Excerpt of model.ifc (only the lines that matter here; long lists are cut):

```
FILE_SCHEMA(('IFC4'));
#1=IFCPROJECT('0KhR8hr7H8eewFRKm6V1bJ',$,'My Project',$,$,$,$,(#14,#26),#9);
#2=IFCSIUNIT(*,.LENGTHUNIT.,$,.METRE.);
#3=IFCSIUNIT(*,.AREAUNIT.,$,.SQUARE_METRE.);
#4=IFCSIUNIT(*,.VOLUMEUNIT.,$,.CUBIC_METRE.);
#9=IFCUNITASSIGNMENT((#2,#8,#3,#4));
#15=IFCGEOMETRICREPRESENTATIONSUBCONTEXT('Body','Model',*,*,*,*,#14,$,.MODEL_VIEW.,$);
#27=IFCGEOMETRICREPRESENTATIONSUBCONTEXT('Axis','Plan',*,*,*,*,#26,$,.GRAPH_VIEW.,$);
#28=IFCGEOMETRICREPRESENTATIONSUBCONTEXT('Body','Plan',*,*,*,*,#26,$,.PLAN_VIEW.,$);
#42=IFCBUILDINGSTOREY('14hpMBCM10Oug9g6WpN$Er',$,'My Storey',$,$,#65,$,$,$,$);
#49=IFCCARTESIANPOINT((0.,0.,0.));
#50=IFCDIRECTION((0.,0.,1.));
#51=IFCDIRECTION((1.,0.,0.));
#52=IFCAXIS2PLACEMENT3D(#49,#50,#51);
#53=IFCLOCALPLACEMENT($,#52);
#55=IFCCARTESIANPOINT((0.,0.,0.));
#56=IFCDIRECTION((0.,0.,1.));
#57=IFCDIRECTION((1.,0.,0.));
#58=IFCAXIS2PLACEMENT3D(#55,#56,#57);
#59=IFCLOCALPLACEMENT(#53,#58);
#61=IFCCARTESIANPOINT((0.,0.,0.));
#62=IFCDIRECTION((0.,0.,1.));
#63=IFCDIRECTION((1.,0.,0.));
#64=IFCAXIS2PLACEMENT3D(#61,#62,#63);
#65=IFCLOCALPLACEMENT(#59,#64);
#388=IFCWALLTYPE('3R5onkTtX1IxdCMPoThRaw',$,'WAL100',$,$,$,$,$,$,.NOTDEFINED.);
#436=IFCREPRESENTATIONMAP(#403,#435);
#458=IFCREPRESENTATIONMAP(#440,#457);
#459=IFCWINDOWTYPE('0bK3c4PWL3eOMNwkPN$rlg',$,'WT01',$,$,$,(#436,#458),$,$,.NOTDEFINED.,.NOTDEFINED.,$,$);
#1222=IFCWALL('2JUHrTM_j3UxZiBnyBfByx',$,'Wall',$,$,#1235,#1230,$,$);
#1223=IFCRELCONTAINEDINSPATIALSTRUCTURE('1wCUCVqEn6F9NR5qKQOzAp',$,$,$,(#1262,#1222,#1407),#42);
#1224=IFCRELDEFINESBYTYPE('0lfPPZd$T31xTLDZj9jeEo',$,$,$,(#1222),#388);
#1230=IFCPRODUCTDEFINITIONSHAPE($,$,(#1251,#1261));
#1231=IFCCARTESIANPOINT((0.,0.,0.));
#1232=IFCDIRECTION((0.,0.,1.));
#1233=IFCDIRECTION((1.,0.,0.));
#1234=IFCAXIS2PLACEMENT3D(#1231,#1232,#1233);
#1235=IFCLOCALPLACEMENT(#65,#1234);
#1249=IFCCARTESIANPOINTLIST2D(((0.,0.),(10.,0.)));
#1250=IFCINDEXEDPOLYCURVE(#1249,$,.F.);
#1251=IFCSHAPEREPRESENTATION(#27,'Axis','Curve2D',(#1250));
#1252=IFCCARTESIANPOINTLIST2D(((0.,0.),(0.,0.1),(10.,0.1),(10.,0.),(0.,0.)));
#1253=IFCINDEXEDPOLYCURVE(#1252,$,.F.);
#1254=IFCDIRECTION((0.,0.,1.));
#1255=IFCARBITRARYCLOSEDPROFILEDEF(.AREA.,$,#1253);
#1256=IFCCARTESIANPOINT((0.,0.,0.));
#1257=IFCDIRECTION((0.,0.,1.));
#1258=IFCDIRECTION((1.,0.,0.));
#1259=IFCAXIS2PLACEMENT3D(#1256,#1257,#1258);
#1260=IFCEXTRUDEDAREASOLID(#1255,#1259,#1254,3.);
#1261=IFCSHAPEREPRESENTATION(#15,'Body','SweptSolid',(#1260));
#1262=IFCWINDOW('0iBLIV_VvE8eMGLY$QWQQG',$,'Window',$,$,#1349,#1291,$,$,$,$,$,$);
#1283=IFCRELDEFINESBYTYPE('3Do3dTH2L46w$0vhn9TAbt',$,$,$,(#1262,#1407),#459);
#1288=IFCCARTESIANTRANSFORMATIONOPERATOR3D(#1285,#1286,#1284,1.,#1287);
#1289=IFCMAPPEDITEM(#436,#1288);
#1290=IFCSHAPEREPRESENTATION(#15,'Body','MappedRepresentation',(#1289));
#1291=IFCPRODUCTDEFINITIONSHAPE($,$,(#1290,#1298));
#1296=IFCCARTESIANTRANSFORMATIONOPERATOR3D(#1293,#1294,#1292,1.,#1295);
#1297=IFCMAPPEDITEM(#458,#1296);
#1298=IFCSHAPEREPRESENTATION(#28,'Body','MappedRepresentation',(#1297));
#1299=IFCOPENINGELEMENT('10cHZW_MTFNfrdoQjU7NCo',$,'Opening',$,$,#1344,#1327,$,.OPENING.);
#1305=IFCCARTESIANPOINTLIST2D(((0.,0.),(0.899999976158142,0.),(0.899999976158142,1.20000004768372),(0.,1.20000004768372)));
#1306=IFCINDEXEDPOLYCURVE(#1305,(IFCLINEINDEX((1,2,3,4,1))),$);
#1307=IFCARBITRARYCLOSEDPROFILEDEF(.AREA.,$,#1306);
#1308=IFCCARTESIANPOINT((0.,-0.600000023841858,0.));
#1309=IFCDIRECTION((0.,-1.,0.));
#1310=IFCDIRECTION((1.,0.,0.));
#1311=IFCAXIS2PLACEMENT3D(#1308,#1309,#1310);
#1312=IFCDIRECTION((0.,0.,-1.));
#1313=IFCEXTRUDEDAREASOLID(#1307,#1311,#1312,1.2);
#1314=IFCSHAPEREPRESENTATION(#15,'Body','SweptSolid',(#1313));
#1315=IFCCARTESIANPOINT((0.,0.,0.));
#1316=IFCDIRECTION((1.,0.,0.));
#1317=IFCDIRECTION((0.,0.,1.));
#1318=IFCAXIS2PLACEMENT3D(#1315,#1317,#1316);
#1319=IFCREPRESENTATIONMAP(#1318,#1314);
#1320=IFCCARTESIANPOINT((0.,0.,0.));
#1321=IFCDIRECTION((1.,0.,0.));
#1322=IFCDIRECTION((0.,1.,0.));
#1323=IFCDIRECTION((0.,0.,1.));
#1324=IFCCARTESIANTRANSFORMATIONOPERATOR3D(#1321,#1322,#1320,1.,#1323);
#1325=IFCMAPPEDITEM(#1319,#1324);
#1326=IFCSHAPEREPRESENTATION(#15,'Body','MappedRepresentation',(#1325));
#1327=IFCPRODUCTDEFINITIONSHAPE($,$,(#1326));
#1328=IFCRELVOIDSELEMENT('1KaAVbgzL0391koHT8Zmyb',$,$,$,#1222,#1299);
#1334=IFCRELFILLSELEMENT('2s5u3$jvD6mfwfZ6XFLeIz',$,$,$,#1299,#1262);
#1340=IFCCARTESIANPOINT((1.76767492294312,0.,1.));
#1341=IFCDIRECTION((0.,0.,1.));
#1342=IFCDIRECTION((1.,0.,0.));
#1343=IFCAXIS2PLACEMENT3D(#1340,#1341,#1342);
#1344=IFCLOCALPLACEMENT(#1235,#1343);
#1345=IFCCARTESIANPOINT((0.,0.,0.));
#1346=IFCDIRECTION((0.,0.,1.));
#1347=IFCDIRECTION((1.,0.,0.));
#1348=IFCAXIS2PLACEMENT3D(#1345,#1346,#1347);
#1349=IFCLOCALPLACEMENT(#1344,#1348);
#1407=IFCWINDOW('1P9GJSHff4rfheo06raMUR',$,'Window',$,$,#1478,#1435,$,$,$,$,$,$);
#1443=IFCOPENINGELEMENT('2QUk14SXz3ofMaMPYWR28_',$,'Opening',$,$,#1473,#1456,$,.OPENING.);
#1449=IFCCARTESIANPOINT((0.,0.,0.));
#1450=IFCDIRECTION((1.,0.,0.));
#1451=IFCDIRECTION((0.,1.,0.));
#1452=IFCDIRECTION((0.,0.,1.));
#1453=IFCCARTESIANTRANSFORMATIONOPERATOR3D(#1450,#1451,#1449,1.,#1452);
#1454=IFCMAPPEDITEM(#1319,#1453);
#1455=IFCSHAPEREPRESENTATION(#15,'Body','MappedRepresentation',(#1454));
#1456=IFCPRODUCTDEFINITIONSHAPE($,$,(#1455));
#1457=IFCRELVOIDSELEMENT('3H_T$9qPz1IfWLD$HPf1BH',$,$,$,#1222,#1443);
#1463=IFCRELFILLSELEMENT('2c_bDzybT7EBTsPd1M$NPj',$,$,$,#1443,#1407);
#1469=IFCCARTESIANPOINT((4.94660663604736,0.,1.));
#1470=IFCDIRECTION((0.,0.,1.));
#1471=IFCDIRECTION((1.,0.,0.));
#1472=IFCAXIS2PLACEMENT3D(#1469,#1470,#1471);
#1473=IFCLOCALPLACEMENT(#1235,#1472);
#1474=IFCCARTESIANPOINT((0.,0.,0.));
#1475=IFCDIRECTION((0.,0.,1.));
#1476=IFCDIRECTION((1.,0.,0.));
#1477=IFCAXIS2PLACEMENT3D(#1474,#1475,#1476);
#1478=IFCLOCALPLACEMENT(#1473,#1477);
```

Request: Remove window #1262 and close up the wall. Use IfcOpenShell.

```python
import ifcopenshell
import ifcopenshell.api.feature
import ifcopenshell.api.root
import ifcopenshell.geom
import ifcopenshell.util.shape

model = ifcopenshell.open("model.ifc")
settings = ifcopenshell.geom.settings()


def volume(element):
    """Net volume in cubic metres, openings subtracted."""
    shape = ifcopenshell.geom.create_shape(settings, element)
    return ifcopenshell.util.shape.get_volume(shape.geometry)


window = model.by_guid("0iBLIV_VvE8eMGLY$QWQQG")
opening = window.FillsVoids[0].RelatingOpeningElement
wall = opening.VoidsElements[0].RelatingBuildingElement
before = volume(wall)

ifcopenshell.api.root.remove_product(model, product=window)
ifcopenshell.api.feature.remove_feature(model, feature=opening)

after = volume(wall)

print(f"wall volume {before:.3f} -> {after:.3f} m3")

model.write("model_updated.ifc")
```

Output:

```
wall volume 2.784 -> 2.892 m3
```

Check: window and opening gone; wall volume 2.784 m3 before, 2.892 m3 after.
